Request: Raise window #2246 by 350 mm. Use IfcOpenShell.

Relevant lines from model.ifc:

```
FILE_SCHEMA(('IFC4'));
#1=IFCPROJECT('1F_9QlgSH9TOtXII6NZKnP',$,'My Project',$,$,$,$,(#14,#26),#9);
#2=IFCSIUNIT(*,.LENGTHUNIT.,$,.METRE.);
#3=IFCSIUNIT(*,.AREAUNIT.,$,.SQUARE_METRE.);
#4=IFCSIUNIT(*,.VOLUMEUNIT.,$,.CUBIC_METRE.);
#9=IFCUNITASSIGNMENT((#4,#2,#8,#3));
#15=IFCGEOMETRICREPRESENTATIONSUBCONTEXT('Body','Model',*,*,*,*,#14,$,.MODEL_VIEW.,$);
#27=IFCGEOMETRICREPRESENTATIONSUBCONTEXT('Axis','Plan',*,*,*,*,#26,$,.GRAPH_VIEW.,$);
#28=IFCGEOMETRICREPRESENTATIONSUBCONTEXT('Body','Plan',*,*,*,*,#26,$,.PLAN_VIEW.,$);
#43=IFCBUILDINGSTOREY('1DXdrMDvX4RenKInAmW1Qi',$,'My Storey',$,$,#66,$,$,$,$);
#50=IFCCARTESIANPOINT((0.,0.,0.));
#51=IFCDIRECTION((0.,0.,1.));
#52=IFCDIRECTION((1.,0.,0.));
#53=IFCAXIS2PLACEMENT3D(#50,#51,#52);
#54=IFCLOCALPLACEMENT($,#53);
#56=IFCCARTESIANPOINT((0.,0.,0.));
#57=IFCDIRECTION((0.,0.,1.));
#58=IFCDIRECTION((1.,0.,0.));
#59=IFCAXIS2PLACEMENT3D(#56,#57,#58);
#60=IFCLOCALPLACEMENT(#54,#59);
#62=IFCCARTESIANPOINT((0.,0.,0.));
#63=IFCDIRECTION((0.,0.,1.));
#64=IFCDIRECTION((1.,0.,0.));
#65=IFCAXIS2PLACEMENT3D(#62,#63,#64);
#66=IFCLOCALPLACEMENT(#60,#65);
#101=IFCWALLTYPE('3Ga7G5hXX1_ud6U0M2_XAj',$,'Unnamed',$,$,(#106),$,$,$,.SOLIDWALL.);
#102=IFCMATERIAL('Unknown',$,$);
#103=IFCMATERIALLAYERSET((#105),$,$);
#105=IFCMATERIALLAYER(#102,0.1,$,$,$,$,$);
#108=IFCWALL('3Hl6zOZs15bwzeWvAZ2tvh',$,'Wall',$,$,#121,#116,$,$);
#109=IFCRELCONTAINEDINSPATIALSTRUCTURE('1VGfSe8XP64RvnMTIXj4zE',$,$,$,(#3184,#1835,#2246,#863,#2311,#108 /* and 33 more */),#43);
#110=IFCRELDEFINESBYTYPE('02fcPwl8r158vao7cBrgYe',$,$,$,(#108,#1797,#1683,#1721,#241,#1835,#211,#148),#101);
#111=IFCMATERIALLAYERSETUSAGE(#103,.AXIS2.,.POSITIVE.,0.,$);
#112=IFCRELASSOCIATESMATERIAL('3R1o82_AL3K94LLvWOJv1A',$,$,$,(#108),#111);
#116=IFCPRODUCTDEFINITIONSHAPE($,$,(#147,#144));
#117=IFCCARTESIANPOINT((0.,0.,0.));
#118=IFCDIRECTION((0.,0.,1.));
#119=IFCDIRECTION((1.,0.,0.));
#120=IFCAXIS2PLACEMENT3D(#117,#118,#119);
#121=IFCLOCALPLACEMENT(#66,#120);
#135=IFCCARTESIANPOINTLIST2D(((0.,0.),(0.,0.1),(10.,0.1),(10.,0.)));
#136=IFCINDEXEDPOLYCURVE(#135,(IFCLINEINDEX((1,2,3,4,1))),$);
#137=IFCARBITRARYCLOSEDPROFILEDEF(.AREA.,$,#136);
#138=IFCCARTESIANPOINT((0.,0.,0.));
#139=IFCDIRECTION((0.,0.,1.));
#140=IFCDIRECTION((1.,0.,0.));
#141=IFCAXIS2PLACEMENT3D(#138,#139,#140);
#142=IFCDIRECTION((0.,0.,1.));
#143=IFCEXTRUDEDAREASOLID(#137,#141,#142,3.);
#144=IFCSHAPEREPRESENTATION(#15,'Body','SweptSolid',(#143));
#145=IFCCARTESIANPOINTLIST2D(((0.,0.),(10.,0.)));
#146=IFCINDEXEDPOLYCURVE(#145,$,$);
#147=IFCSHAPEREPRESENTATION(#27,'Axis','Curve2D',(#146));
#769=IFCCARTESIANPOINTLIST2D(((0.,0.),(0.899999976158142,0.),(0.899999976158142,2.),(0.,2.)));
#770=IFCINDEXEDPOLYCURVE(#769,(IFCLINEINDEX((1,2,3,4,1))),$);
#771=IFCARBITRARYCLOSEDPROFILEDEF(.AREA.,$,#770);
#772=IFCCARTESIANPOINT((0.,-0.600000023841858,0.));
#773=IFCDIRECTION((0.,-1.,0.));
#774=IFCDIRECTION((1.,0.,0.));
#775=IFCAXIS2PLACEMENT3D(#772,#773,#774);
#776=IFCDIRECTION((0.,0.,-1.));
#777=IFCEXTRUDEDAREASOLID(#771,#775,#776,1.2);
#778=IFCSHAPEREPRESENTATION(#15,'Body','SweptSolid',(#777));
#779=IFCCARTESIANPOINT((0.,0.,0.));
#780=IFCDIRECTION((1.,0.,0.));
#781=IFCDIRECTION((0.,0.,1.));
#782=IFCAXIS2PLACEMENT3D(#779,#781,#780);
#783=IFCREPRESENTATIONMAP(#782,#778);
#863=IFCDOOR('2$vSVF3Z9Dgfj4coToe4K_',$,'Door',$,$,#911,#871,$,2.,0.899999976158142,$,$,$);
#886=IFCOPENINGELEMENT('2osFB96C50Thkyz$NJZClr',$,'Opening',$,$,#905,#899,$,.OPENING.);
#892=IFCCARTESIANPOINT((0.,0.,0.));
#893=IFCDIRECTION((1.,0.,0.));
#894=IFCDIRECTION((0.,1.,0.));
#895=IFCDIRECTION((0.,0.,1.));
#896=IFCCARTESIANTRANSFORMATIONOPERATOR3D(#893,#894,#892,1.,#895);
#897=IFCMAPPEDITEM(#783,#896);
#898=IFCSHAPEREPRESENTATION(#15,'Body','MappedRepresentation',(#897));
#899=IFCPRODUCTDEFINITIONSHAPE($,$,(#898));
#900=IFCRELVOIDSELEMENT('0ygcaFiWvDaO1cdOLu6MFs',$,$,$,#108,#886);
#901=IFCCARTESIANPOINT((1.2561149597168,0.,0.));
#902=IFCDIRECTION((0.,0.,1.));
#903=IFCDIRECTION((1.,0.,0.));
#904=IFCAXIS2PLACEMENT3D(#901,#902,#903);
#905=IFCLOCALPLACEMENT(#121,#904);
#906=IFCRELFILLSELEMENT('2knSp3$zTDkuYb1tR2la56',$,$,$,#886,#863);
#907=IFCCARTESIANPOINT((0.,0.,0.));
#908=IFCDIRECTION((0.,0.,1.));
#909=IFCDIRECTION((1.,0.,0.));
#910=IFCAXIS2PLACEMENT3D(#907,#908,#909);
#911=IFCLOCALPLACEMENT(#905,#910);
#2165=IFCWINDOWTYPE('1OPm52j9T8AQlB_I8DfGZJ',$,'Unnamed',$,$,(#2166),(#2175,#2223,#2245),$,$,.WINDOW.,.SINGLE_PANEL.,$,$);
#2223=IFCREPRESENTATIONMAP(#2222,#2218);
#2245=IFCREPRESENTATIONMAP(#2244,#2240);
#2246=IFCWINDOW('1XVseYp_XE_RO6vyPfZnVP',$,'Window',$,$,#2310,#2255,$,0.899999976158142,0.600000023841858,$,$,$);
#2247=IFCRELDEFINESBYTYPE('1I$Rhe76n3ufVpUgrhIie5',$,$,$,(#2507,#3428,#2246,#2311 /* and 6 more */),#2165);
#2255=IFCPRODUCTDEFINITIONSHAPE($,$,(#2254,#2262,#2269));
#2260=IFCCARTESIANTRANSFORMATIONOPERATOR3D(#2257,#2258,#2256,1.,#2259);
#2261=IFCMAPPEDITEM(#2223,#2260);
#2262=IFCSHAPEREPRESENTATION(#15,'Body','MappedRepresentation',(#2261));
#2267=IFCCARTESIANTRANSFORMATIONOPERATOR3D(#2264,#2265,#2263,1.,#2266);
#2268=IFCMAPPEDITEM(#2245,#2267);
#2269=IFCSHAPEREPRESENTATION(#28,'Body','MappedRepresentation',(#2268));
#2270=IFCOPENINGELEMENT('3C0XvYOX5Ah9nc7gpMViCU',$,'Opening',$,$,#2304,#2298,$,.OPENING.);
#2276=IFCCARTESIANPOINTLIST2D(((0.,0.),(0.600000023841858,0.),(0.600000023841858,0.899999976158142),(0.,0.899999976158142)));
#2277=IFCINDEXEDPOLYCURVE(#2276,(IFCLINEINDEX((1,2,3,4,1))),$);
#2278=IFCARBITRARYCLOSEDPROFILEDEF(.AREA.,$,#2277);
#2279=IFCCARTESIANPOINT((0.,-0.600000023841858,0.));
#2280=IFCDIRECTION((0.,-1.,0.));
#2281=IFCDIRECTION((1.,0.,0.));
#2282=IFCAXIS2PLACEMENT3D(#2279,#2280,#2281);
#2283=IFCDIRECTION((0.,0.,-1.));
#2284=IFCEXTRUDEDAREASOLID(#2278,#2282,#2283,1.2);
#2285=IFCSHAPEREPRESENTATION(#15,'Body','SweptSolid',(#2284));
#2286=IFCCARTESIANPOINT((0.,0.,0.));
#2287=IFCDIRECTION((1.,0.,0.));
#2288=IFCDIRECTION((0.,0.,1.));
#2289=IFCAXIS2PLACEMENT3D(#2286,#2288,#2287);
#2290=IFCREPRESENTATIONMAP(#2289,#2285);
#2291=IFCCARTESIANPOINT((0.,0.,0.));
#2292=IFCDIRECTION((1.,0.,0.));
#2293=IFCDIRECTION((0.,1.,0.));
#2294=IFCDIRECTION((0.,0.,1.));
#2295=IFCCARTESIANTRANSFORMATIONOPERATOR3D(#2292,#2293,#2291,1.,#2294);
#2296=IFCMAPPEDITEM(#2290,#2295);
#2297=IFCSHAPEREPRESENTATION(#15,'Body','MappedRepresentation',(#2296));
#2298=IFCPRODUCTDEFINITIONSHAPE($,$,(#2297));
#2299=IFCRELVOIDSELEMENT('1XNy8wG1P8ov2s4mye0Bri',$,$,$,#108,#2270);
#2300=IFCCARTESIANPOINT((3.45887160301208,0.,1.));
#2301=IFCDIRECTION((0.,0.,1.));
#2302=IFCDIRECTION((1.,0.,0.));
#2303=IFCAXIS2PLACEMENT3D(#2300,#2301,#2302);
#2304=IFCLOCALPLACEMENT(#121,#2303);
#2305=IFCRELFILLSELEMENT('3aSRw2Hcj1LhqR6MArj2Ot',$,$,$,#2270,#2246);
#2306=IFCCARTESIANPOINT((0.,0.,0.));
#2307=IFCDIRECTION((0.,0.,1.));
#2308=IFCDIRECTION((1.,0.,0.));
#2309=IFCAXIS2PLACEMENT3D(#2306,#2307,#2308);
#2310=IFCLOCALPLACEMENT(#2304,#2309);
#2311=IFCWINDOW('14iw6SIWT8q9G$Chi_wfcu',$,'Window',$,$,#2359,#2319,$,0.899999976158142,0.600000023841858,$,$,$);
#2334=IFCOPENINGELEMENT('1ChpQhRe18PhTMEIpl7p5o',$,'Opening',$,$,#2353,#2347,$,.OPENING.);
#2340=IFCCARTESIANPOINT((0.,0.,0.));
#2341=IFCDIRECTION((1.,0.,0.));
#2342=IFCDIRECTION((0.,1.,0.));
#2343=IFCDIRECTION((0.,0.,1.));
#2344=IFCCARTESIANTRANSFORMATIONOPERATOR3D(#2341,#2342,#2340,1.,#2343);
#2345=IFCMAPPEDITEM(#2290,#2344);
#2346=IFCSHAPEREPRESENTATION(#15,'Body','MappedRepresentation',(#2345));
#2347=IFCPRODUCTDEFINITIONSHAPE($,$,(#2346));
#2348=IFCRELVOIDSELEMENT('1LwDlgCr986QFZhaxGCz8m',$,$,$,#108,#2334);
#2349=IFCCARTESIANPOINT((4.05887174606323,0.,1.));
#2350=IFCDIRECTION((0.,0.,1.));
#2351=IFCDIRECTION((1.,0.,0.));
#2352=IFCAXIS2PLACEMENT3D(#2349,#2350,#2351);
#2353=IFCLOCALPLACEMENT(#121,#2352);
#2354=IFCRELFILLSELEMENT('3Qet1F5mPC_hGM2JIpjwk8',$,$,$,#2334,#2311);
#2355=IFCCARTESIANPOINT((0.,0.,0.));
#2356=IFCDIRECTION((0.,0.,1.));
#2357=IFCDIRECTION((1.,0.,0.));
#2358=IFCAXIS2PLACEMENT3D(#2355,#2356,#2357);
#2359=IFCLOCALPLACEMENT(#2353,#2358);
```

```python
import numpy as np
import ifcopenshell
import ifcopenshell.api.geometry
import ifcopenshell.util.placement
import ifcopenshell.util.unit

model = ifcopenshell.open("model.ifc")
unit_scale = ifcopenshell.util.unit.calculate_unit_scale(model)

window = model.by_guid("1XVseYp_XE_RO6vyPfZnVP")
opening = window.FillsVoids[0].RelatingOpeningElement
dz = 0.35 / unit_scale

shift = np.array([0.0, 0.0, dz])
# The window is placed relative to its opening, so it follows when the opening moves.
matrix = ifcopenshell.util.placement.get_local_placement(opening.ObjectPlacement)
matrix[:3, 3] += shift
ifcopenshell.api.geometry.edit_object_placement(
    model, product=opening, matrix=matrix, is_si=False, should_transform_children=True
)

print(f"moved by {dz * unit_scale:+.3f} m")

model.write("model-out.ifc")
```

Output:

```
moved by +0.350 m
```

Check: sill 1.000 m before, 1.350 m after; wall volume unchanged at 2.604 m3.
